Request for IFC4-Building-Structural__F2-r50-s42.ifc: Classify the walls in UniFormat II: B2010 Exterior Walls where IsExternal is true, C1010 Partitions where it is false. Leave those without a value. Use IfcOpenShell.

First a look at what the model holds.

```python
import ifcopenshell
import ifcopenshell.util.element

model = ifcopenshell.open("IFC4-Building-Structural__F2-r50-s42.ifc")
print(model.schema)
print("classifications:", [c.Name for c in model.by_type("IfcClassification")])
values = [ifcopenshell.util.element.get_pset(e, "Pset_WallCommon", "IsExternal") for e in model.by_type("IfcWall")]
for value in (True, False, None):
    print("IsExternal", value, values.count(value))
```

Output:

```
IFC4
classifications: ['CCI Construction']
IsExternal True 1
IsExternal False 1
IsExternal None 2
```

```python
import ifcopenshell
import ifcopenshell.api.classification
import ifcopenshell.util.element

model = ifcopenshell.open("IFC4-Building-Structural__F2-r50-s42.ifc")

system = ifcopenshell.api.classification.add_classification(model, classification="UniFormat II")

walls = model.by_type("IfcWall")
external = {e: ifcopenshell.util.element.get_pset(e, "Pset_WallCommon", "IsExternal") for e in walls}
for flag, code, name in ((True, "B2010", "Exterior Walls"), (False, "C1010", "Partitions")):
    products = [e for e in walls if external[e] is flag]
    ifcopenshell.api.classification.add_reference(
        model, products=products, classification=system, identification=code, name=name
    )
    print(code, len(products))

model.write("IFC4-Building-Structural__F2-r50-s42_edited.ifc")
```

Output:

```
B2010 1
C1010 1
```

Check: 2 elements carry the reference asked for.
